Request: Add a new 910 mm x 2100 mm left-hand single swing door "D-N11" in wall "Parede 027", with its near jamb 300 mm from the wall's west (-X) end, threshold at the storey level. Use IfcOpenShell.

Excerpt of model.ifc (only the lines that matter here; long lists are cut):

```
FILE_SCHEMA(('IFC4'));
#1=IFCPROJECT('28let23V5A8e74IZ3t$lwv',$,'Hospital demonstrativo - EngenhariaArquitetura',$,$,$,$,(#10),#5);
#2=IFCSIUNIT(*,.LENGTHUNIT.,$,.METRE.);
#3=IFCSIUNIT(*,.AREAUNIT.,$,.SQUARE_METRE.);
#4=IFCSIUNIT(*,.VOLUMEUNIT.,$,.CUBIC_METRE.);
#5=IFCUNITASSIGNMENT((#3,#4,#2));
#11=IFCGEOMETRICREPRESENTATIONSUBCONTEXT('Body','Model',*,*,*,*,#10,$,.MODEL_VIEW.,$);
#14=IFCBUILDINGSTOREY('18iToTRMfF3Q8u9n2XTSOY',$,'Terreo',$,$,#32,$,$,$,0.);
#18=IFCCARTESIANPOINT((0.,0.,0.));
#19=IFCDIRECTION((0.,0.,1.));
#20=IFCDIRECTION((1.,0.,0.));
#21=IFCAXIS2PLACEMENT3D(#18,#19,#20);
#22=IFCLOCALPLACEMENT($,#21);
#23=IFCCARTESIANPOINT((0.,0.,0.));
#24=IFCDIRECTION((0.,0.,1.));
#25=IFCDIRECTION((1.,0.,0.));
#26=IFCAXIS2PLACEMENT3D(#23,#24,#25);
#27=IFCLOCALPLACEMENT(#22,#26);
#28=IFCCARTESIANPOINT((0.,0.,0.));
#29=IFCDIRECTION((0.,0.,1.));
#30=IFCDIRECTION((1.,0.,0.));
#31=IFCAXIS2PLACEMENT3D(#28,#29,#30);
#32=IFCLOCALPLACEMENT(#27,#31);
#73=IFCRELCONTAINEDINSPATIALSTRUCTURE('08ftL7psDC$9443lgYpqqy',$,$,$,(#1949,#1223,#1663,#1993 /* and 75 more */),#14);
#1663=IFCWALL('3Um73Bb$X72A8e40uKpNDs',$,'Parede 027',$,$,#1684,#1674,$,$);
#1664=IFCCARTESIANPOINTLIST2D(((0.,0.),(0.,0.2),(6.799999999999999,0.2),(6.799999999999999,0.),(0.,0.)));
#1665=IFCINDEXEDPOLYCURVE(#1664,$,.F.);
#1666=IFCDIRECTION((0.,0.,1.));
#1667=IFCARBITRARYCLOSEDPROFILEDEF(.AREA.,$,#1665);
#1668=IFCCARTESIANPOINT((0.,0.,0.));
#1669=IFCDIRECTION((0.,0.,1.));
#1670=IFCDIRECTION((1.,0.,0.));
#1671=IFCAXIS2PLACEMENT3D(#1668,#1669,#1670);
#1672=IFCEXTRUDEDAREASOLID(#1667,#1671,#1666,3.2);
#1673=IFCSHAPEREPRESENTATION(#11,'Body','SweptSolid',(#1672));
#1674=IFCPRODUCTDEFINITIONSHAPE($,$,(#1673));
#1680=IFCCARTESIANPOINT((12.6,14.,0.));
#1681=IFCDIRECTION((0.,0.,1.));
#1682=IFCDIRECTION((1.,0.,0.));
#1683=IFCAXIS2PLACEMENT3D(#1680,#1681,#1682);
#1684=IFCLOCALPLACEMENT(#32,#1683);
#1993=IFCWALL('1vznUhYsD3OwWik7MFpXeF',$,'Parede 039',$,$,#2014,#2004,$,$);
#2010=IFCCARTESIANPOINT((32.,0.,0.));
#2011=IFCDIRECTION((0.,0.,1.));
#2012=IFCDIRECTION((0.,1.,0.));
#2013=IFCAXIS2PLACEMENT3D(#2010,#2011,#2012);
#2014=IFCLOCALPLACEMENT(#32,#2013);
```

```python
import numpy as np
import ifcopenshell
import ifcopenshell.api.feature
import ifcopenshell.api.geometry
import ifcopenshell.api.root
import ifcopenshell.api.spatial
import ifcopenshell.geom
import ifcopenshell.util.element
import ifcopenshell.util.placement
import ifcopenshell.util.representation
import ifcopenshell.util.shape
import ifcopenshell.util.unit

model = ifcopenshell.open("model.ifc")
unit_scale = ifcopenshell.util.unit.calculate_unit_scale(model)
settings = ifcopenshell.geom.settings()


def volume(element):
    """Net volume in cubic metres, openings subtracted."""
    shape = ifcopenshell.geom.create_shape(settings, element)
    return ifcopenshell.util.shape.get_volume(shape.geometry)


wall = model.by_id(1663)
storey = ifcopenshell.util.element.get_container(wall, ifc_class="IfcBuildingStorey")
context = ifcopenshell.util.representation.get_context(model, "Model", "Body", "MODEL_VIEW")
before = volume(wall)

width, height, from_end, sill = 0.91, 2.1, 0.3, 0.0  # metres

# The wall runs along its own X axis, and the end named is its -X end.
wall_shape = ifcopenshell.geom.create_shape(settings, wall)
x, y, z = ifcopenshell.util.shape.get_vertices(wall_shape.geometry).T
start = x.min() + from_end
face, thickness = float(y.min()), float(y.max() - y.min())
wall_matrix = ifcopenshell.util.placement.get_local_placement(wall.ObjectPlacement)
level = ifcopenshell.util.placement.get_local_placement(storey.ObjectPlacement)[2, 3]


def in_wall(x, y):
    """Placement at x, y metres in the wall's axes, at sill height."""
    matrix = wall_matrix.copy()
    matrix[:, 3] = wall_matrix @ np.array([x / unit_scale, y / unit_scale, 0.0, 1.0])
    matrix[2, 3] = level + sill / unit_scale
    return matrix


# Opening: a box that overshoots both wall faces by 50 mm.
opening = ifcopenshell.api.root.create_entity(model, ifc_class="IfcOpeningElement", predefined_type="OPENING")
box = ifcopenshell.api.geometry.add_wall_representation(
    model, context=context, length=width, height=height, thickness=thickness + 0.1
)
ifcopenshell.api.geometry.assign_representation(model, product=opening, representation=box)
ifcopenshell.api.geometry.edit_object_placement(model, product=opening, matrix=in_wall(start, face - 0.05), is_si=False)
ifcopenshell.api.feature.add_feature(model, feature=opening, element=wall)

door = ifcopenshell.api.root.create_entity(model, ifc_class="IfcDoor", name="D-N11", predefined_type="DOOR")
door.OverallWidth, door.OverallHeight = width / unit_scale, height / unit_scale
door.OperationType = "SINGLE_SWING_LEFT"
body = ifcopenshell.api.geometry.add_door_representation(
    model,
    context=context,
    overall_width=door.OverallWidth,
    overall_height=door.OverallHeight,
    operation_type="SINGLE_SWING_LEFT",
    lining_properties={"LiningDepth": thickness / unit_scale, "ThresholdDepth": thickness / unit_scale},
)
ifcopenshell.api.geometry.assign_representation(model, product=door, representation=body)
ifcopenshell.api.spatial.assign_container(model, products=[door], relating_structure=storey)
ifcopenshell.api.feature.add_filling(model, opening=opening, element=door)

# The lining spans the wall, so the door starts at the wall face.
ifcopenshell.api.geometry.edit_object_placement(model, product=door, matrix=in_wall(start, face), is_si=False)

after = volume(wall)

print(f"wall volume {before:.3f} -> {after:.3f} m3")

model.write("model_v2.ifc")
```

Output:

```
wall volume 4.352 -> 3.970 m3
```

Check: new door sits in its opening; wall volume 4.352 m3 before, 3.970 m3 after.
